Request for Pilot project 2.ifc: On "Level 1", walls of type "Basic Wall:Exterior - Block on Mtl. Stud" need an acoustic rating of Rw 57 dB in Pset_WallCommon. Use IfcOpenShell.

First a look at what the model holds.

```python
import ifcopenshell
import ifcopenshell.util.element

model = ifcopenshell.open("Pilot project 2.ifc")
print(model.schema)
storey = next(s for s in model.by_type("IfcBuildingStorey") if s.Name == "Level 1")
walls = [e for e in ifcopenshell.util.element.get_decomposition(storey) if e.is_a("IfcWall")]
seen = {}
for e in walls:
    element_type = ifcopenshell.util.element.get_type(e)
    key = (element_type.Name if element_type != e and element_type else None, ifcopenshell.util.element.get_pset(e, "Pset_WallCommon", "AcousticRating"))
    seen[key] = seen.get(key, 0) + 1
for (name, value), count in sorted(seen.items(), key=str):
    print(count, "x", name, "|", value)
```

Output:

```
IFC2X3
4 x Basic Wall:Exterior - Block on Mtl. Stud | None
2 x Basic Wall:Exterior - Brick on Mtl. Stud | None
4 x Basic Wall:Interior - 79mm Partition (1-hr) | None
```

```python
import ifcopenshell
import ifcopenshell.api.pset
import ifcopenshell.util.element

model = ifcopenshell.open("Pilot project 2.ifc")

storey = next(s for s in model.by_type("IfcBuildingStorey") if s.Name == "Level 1")
walls = [e for e in ifcopenshell.util.element.get_decomposition(storey) if e.is_a("IfcWall")]

count = 0
for e in walls:
    element_type = ifcopenshell.util.element.get_type(e)
    if element_type in (None, e) or element_type.Name != "Basic Wall:Exterior - Block on Mtl. Stud":
        continue
    # add_pset returns the element's existing set when there is one.
    pset = ifcopenshell.api.pset.add_pset(model, product=e, name="Pset_WallCommon")
    ifcopenshell.api.pset.edit_pset(model, pset=pset, properties={"AcousticRating": "Rw 57 dB"})
    count += 1

print(count, "walls updated")

model.write("Pilot project 2_rev.ifc")
```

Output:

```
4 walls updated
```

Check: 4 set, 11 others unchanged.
